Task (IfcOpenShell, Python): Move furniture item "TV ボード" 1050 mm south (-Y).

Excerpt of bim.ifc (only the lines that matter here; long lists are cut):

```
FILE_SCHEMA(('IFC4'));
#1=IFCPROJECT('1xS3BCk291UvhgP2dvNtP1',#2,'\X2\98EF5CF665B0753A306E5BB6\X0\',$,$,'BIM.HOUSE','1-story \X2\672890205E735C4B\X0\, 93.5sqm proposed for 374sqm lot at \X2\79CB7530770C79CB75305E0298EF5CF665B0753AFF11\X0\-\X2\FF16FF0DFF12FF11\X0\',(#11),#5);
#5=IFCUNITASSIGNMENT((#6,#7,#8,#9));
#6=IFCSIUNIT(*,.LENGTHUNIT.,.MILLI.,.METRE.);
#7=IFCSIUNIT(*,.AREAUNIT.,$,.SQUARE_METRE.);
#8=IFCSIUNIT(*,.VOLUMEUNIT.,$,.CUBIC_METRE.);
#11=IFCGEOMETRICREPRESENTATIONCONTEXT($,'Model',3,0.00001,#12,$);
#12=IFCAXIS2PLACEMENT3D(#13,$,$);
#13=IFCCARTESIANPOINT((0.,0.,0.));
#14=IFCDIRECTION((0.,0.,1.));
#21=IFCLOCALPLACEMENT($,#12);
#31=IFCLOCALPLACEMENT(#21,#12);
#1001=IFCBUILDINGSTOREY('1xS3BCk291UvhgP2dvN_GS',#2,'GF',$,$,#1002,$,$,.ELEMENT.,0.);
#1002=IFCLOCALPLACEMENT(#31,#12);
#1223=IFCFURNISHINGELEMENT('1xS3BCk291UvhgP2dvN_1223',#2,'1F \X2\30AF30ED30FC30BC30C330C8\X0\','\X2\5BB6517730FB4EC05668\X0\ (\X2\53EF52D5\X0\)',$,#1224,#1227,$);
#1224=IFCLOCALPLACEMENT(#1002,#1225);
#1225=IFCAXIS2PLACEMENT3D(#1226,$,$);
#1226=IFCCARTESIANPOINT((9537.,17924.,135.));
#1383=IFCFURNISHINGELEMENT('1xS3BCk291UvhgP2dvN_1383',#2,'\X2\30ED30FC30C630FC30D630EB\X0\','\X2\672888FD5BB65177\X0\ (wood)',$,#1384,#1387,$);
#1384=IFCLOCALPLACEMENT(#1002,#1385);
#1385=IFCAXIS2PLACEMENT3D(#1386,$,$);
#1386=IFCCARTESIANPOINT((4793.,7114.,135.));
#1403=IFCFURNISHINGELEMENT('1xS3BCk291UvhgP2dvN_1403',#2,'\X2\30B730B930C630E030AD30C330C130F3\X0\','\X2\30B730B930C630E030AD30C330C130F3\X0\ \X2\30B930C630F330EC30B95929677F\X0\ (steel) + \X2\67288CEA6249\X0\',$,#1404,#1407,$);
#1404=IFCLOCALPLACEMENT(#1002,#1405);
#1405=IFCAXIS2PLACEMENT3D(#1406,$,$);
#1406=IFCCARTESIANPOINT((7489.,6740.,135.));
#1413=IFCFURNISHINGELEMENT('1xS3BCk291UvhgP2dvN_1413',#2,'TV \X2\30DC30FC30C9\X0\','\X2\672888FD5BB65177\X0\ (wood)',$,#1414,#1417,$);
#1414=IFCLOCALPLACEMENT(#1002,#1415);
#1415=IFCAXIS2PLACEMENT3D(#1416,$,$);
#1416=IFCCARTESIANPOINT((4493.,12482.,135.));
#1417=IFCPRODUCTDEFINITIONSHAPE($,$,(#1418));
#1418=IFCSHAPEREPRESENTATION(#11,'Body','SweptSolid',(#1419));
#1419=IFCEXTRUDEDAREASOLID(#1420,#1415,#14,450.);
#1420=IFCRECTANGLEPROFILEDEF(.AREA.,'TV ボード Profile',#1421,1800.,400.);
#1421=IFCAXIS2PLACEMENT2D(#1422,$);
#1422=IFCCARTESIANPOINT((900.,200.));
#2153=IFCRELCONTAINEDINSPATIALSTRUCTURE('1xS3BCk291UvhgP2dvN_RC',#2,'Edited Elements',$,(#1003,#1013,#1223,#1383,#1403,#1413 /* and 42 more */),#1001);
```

```python
import ifcopenshell
import ifcopenshell.api.geometry
import ifcopenshell.util.placement
import ifcopenshell.util.unit

model = ifcopenshell.open("bim.ifc")
unit_scale = ifcopenshell.util.unit.calculate_unit_scale(model)

item = model.by_guid("1xS3BCk291UvhgP2dvN_1413")
matrix = ifcopenshell.util.placement.get_local_placement(item.ObjectPlacement)
matrix[1, 3] -= 1.05 / unit_scale
ifcopenshell.api.geometry.edit_object_placement(model, product=item, matrix=matrix, is_si=False)

print(ifcopenshell.util.placement.get_local_placement(item.ObjectPlacement).round(3) + 0.0)

model.write("bim_v2.ifc")
```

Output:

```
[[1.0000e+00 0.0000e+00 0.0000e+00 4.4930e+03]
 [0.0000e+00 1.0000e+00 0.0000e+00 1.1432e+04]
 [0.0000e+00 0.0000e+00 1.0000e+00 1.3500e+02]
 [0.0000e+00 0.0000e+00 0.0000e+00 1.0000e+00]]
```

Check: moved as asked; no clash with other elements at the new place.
